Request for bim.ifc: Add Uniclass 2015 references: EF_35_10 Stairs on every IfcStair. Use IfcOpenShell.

First a look at what the model holds.

```python
import ifcopenshell

model = ifcopenshell.open("bim.ifc")
print(model.schema)
print("classifications:", [c.Name for c in model.by_type("IfcClassification")])
for ifc_class in ("IfcDoor", "IfcRoof", "IfcStair", "IfcWall", "IfcWindow"):
    print(ifc_class, len(model.by_type(ifc_class)))
```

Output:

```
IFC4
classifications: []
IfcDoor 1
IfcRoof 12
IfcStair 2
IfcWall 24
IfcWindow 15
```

```python
import ifcopenshell
import ifcopenshell.api.classification

model = ifcopenshell.open("bim.ifc")

system = ifcopenshell.api.classification.add_classification(model, classification="Uniclass 2015")

codes = {
    "IfcStair": ("EF_35_10", "Stairs"),
}
for ifc_class, (code, name) in codes.items():
    products = model.by_type(ifc_class)
    ifcopenshell.api.classification.add_reference(
        model, products=products, classification=system, identification=code, name=name
    )
    print(code, len(products))

model.write("bim_rev.ifc")
```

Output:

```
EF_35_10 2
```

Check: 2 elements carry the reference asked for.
